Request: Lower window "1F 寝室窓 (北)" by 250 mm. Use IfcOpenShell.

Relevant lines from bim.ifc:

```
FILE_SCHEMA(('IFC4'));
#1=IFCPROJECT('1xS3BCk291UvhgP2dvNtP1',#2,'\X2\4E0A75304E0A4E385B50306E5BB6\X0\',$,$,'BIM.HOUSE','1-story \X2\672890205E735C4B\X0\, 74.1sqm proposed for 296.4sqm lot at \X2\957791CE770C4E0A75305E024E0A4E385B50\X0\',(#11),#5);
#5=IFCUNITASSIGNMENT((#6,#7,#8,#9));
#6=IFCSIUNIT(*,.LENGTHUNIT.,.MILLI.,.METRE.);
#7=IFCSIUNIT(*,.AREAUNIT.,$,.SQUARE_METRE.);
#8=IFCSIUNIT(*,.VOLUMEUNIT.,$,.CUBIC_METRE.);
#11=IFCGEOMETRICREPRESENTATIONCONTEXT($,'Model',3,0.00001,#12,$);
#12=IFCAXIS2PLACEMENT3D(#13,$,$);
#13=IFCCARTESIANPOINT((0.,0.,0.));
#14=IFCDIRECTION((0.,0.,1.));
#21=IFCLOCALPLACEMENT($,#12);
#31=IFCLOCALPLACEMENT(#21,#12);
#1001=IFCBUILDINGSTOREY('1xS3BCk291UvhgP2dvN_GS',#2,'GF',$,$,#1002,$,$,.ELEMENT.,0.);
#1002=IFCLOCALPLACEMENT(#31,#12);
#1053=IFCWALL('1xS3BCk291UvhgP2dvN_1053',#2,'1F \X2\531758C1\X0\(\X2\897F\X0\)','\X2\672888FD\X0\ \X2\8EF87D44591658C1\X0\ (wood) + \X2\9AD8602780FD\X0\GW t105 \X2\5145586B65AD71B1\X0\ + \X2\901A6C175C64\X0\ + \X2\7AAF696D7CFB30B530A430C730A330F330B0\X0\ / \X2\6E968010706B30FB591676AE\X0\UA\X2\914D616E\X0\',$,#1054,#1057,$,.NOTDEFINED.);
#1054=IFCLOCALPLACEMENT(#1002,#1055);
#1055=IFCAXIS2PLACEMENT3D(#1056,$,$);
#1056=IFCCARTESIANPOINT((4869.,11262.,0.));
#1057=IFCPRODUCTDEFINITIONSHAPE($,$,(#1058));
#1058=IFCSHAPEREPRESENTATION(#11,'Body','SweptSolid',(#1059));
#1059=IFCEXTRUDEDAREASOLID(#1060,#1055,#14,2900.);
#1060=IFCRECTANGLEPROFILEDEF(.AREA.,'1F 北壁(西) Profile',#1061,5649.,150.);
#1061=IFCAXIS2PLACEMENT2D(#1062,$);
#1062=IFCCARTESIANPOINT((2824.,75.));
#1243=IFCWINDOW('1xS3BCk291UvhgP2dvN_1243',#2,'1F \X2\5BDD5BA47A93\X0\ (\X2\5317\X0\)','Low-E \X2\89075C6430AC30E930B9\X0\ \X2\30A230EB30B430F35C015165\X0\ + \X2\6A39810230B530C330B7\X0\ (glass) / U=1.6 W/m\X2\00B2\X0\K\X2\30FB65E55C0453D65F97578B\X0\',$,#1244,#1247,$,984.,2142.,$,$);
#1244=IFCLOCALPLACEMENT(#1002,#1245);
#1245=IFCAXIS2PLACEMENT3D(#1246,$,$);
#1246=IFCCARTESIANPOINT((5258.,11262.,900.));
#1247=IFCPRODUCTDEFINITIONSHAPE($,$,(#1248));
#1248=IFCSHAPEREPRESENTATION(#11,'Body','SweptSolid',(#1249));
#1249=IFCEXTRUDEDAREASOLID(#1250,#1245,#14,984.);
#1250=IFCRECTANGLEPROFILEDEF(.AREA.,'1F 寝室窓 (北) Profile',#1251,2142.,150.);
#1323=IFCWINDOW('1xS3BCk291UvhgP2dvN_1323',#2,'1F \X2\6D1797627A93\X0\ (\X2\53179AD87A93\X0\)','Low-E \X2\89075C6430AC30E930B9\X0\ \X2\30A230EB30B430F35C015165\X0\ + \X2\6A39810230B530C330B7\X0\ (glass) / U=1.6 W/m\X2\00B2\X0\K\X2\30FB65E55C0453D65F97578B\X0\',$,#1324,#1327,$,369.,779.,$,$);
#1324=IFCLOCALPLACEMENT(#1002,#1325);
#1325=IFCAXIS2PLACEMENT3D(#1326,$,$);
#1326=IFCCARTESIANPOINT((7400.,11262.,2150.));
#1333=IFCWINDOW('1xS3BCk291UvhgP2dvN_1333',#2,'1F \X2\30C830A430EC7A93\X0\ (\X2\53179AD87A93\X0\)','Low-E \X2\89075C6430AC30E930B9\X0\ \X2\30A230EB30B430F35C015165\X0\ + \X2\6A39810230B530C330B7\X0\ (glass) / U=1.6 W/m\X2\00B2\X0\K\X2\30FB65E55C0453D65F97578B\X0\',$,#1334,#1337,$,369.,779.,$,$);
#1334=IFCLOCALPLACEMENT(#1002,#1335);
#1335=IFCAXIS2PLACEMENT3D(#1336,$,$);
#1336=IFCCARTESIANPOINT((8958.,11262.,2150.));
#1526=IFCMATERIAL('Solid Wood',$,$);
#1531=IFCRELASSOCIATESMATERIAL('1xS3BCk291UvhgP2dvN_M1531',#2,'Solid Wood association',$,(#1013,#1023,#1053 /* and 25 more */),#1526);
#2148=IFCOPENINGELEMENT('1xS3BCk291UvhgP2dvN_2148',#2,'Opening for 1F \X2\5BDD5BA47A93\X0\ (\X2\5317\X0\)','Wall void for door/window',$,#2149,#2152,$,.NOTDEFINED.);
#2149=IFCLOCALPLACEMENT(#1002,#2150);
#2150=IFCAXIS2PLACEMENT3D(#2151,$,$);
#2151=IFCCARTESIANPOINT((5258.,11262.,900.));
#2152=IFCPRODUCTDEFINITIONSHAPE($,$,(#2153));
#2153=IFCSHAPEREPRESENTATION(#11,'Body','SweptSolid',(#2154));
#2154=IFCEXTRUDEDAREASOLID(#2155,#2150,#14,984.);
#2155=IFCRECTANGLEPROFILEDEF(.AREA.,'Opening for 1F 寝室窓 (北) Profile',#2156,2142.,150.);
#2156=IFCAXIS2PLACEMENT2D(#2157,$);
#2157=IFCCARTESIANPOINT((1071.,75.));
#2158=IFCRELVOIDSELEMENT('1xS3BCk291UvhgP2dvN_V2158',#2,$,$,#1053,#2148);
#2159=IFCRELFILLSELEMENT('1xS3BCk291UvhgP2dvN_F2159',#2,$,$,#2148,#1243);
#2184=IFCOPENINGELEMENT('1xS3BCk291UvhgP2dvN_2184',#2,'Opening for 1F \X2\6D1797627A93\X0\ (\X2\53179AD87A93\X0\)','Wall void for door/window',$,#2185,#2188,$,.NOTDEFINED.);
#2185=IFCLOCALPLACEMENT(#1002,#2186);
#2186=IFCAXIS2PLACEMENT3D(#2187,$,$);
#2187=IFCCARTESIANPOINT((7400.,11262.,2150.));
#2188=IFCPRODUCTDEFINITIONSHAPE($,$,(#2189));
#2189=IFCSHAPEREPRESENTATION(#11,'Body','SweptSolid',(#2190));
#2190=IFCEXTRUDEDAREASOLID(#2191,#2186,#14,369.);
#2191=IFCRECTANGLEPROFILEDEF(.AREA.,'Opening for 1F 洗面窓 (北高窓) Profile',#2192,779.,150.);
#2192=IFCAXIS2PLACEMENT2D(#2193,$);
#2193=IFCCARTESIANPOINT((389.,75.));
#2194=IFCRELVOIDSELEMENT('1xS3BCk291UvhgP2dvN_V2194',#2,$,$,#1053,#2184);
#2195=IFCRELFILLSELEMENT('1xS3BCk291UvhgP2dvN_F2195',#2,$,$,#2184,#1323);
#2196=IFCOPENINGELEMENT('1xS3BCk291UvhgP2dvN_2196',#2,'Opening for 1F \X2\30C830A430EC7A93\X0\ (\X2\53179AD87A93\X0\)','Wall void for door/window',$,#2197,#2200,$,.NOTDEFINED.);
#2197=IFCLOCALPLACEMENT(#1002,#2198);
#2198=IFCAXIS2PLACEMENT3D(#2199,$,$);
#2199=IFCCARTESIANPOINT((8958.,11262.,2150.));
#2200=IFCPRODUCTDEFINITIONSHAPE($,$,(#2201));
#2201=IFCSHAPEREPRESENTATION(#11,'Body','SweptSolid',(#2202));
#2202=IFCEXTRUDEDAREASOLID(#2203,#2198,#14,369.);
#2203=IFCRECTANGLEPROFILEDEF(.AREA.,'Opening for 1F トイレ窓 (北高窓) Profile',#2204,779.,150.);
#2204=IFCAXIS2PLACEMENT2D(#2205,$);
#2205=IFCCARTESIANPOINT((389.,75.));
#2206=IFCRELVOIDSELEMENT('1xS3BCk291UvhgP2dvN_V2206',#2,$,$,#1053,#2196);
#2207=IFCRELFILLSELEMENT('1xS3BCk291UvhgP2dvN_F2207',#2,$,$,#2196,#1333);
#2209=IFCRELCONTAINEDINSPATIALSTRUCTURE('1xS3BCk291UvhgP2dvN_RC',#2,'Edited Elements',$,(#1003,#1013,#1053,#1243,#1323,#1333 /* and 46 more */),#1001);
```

```python
import numpy as np
import ifcopenshell
import ifcopenshell.api.geometry
import ifcopenshell.util.placement
import ifcopenshell.util.unit

model = ifcopenshell.open("bim.ifc")
unit_scale = ifcopenshell.util.unit.calculate_unit_scale(model)

window = model.by_guid("1xS3BCk291UvhgP2dvN_1243")
opening = window.FillsVoids[0].RelatingOpeningElement
dz = -250.0

shift = np.array([0.0, 0.0, dz])
# The window is not placed relative to its opening, so move both.
for product in (opening, window):
    matrix = ifcopenshell.util.placement.get_local_placement(product.ObjectPlacement)
    matrix[:3, 3] += shift
    ifcopenshell.api.geometry.edit_object_placement(model, product=product, matrix=matrix, is_si=False)

print(f"moved by {dz * unit_scale:+.3f} m")

model.write("bim_rev.ifc")
```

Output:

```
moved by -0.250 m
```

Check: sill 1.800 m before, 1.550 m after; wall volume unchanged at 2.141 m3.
